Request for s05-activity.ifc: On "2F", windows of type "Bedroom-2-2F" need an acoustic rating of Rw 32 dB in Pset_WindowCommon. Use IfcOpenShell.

First a look at what the model holds.

```python
import ifcopenshell
import ifcopenshell.util.element

model = ifcopenshell.open("s05-activity.ifc")
print(model.schema)
storey = next(s for s in model.by_type("IfcBuildingStorey") if s.Name == "2F")
windows = [e for e in ifcopenshell.util.element.get_decomposition(storey) if e.is_a("IfcWindow")]
seen = {}
for e in windows:
    element_type = ifcopenshell.util.element.get_type(e)
    key = (element_type.Name if element_type != e and element_type else None, ifcopenshell.util.element.get_pset(e, "Pset_WindowCommon", "AcousticRating"))
    seen[key] = seen.get(key, 0) + 1
for (name, value), count in sorted(seen.items(), key=str):
    print(count, "x", name, "|", value)
```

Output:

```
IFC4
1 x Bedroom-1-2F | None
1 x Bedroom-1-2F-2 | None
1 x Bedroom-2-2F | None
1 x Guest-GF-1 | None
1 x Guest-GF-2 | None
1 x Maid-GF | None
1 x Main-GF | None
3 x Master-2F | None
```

```python
import ifcopenshell
import ifcopenshell.api.pset
import ifcopenshell.util.element

model = ifcopenshell.open("s05-activity.ifc")

storey = next(s for s in model.by_type("IfcBuildingStorey") if s.Name == "2F")
windows = [e for e in ifcopenshell.util.element.get_decomposition(storey) if e.is_a("IfcWindow")]

count = 0
for e in windows:
    element_type = ifcopenshell.util.element.get_type(e)
    if element_type in (None, e) or element_type.Name != "Bedroom-2-2F":
        continue
    # add_pset returns the element's existing set when there is one.
    pset = ifcopenshell.api.pset.add_pset(model, product=e, name="Pset_WindowCommon")
    ifcopenshell.api.pset.edit_pset(model, pset=pset, properties={"AcousticRating": "Rw 32 dB"})
    count += 1

print(count, "windows updated")

model.write("s05-activity_edited.ifc")
```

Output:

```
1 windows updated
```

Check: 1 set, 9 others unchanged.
